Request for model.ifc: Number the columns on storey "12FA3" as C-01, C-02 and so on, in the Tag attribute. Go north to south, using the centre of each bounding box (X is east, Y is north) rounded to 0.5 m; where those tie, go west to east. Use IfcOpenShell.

First a look at what the model holds.

```python
import ifcopenshell
import ifcopenshell.util.element
import ifcopenshell.util.placement

model = ifcopenshell.open("model.ifc")
print(model.schema)
storey = next(s for s in model.by_type("IfcBuildingStorey") if s.Name == "12FA3")
columns = [e for e in ifcopenshell.util.element.get_decomposition(storey) if e.is_a("IfcColumn")]
for e in sorted(columns, key=lambda e: e.id()):
    origin = ifcopenshell.util.placement.get_local_placement(e.ObjectPlacement)[:3, 3]
    print(e.id(), e.Tag, e.Name, origin.round(2) + 0.0, sep=" | ")
```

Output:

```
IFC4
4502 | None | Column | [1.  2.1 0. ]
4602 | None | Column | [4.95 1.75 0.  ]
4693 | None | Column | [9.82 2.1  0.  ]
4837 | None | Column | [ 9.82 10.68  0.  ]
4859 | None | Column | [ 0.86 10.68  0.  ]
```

```python
import ifcopenshell
import ifcopenshell.geom
import ifcopenshell.util.element
import ifcopenshell.util.shape

model = ifcopenshell.open("model.ifc")
settings = ifcopenshell.geom.settings()
settings.set("use-world-coords", True)


def centre(element):
    shape = ifcopenshell.geom.create_shape(settings, element)
    return ifcopenshell.util.shape.get_bbox_centroid(shape.geometry)


storey = next(s for s in model.by_type("IfcBuildingStorey") if s.Name == "12FA3")
columns = [e for e in ifcopenshell.util.element.get_decomposition(storey) if e.is_a("IfcColumn")]

# Insertion points can sit at a corner or the storey origin, so sort by the geometry (in metres).
centres = {e: centre(e) for e in columns}
columns.sort(key=lambda e: (-round(centres[e][1] / 0.5), centres[e][0]))

for i, e in enumerate(columns, start=1):
    number = f"C-{i:02d}"
    e.Tag = number
    print(e.id(), number)

model.write("model_v2.ifc")
```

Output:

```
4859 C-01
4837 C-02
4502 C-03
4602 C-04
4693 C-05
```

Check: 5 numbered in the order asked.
